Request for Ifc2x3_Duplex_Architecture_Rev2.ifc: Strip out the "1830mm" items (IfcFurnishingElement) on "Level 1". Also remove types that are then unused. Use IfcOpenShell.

First a look at what the model holds.

```python
import ifcopenshell
import ifcopenshell.util.element

model = ifcopenshell.open("Ifc2x3_Duplex_Architecture_Rev2.ifc")
print(model.schema)
storey = next(s for s in model.by_type("IfcBuildingStorey") if s.Name == "Level 1")
furniture = [e for e in ifcopenshell.util.element.get_decomposition(storey) if e.is_a("IfcFurnishingElement")]
seen = {}
for e in furniture:
    element_type = ifcopenshell.util.element.get_type(e)
    name = element_type.Name if element_type not in (None, e) else None
    seen[name] = seen.get(name, 0) + 1
for name, count in sorted(seen.items(), key=str):
    print(count, "x", name)
```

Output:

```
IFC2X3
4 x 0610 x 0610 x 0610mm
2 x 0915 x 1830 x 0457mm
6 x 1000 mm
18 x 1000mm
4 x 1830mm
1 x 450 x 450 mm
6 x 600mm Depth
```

```python
import ifcopenshell
import ifcopenshell.api.root
import ifcopenshell.util.element

model = ifcopenshell.open("Ifc2x3_Duplex_Architecture_Rev2.ifc")

storey = next(s for s in model.by_type("IfcBuildingStorey") if s.Name == "Level 1")
furniture = [e for e in ifcopenshell.util.element.get_decomposition(storey) if e.is_a("IfcFurnishingElement")]
targets = [e for e in furniture if (t := ifcopenshell.util.element.get_type(e)) not in (None, e) and t.Name == "1830mm"]
types = {ifcopenshell.util.element.get_type(e) for e in targets} - {None, *targets}

for e in targets:
    ifcopenshell.api.root.remove_product(model, product=e)
print(len(targets), "removed")

unused = [t for t in types if not ifcopenshell.util.element.get_types(t)]
for t in unused:
    ifcopenshell.api.root.remove_product(model, product=t)
print(len(unused), "unused types removed")

model.write("Ifc2x3_Duplex_Architecture_Rev2-out.ifc")
```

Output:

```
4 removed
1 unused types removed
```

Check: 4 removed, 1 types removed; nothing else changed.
